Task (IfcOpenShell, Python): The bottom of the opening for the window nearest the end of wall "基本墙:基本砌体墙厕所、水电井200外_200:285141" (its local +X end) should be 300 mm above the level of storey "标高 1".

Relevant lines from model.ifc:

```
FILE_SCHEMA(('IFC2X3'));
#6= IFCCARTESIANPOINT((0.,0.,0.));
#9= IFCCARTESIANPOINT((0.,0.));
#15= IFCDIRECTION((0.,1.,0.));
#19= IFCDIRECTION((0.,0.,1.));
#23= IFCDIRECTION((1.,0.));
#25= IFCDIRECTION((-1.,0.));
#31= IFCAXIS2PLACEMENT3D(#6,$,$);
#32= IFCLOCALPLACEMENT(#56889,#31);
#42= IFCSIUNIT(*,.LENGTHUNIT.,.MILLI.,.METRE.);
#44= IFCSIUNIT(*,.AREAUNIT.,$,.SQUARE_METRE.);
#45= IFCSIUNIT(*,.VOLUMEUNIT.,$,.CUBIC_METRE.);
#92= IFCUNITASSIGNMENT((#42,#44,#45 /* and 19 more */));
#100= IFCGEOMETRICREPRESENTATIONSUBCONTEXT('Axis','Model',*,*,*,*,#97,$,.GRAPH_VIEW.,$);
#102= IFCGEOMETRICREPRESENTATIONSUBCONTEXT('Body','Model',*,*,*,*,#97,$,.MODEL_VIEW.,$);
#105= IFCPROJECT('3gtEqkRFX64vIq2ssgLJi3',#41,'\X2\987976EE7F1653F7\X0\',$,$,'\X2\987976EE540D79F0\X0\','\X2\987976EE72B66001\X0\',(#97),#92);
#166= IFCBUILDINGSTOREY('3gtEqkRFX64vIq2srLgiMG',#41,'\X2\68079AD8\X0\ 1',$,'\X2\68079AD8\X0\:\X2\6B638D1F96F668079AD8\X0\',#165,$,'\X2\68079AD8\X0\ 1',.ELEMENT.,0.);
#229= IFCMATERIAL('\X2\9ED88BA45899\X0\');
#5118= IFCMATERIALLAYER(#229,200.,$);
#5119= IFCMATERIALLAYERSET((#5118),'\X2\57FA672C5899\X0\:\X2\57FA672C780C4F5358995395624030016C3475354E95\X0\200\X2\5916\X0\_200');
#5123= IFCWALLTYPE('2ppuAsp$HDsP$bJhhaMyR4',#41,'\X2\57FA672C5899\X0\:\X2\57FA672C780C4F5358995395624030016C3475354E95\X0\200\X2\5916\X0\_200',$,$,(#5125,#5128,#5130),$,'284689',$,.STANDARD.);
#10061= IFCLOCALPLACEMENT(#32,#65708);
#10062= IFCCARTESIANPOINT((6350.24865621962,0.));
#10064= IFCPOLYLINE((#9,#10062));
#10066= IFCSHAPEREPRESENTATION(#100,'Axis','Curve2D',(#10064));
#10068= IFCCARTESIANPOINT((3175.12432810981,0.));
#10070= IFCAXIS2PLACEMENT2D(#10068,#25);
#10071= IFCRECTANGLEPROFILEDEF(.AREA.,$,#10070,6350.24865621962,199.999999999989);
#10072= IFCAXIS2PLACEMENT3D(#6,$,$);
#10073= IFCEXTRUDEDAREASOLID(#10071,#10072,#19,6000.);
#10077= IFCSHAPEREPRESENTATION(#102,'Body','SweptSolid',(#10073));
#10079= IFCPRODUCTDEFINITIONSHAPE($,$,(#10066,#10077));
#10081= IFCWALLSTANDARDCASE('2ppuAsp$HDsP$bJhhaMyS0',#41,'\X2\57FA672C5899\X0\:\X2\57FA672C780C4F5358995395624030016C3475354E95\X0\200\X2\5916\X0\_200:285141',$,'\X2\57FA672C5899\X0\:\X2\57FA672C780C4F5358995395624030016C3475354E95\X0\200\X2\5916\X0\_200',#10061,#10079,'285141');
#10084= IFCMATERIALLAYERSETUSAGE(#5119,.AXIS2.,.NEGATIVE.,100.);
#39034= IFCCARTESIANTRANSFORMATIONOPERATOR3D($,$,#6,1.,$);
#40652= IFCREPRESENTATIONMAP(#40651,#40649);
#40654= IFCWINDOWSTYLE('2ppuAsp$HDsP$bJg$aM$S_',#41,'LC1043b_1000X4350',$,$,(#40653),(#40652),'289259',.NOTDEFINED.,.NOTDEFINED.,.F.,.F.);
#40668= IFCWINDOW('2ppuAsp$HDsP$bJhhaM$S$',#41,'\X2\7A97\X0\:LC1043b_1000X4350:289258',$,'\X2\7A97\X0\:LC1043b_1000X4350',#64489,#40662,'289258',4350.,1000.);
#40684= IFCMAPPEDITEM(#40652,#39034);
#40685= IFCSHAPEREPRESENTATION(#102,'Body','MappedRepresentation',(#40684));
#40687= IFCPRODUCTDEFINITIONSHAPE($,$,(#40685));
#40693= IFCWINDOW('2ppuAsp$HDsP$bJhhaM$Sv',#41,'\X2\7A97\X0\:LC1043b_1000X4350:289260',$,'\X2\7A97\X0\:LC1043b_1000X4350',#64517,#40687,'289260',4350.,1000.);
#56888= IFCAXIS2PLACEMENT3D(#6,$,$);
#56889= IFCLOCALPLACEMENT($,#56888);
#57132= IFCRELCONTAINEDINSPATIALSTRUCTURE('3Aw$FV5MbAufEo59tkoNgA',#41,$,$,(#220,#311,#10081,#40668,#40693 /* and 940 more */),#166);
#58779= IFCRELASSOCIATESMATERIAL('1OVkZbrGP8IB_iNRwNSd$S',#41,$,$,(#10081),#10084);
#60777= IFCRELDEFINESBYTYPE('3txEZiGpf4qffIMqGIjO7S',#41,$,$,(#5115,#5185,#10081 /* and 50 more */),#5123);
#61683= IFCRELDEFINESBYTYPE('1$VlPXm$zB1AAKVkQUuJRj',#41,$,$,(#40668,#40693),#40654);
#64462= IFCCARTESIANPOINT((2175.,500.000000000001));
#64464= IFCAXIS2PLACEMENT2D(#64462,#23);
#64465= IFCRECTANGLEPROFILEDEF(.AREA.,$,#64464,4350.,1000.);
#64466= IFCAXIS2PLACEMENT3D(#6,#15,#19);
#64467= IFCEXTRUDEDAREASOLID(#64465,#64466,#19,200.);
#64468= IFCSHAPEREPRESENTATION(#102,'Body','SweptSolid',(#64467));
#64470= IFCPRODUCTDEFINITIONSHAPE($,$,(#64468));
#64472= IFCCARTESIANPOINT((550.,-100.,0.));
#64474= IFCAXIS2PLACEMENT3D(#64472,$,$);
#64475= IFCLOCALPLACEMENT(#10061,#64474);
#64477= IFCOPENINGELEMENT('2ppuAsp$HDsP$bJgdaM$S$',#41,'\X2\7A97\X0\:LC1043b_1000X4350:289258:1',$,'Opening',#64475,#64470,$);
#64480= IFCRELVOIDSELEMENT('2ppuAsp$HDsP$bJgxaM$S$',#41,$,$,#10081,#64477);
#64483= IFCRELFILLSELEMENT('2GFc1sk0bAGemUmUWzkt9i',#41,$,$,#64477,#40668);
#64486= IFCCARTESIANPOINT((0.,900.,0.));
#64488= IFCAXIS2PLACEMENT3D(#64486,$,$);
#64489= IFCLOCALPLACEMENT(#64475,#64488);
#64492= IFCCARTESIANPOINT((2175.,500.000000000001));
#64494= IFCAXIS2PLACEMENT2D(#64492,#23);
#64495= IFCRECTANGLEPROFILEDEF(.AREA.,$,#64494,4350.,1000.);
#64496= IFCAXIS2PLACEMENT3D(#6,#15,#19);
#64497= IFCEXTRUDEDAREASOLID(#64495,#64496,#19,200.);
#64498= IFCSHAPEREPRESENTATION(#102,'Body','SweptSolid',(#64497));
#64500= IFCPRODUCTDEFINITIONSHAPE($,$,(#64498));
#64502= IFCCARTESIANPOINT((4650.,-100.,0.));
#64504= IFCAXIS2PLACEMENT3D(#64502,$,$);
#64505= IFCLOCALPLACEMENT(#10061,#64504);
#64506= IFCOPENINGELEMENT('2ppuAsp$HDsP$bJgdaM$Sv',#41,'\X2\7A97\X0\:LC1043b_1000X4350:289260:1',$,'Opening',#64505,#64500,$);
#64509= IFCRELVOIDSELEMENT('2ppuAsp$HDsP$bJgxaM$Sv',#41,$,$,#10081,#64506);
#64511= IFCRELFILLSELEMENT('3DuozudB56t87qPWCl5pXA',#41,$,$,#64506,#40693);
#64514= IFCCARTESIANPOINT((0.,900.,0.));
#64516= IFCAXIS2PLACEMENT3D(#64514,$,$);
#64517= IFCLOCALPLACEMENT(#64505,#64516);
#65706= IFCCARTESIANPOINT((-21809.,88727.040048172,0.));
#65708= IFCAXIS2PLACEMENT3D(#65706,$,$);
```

```python
import numpy as np
import ifcopenshell
import ifcopenshell.api.geometry
import ifcopenshell.geom
import ifcopenshell.util.element
import ifcopenshell.util.placement
import ifcopenshell.util.shape
import ifcopenshell.util.unit

model = ifcopenshell.open("model.ifc")
unit_scale = ifcopenshell.util.unit.calculate_unit_scale(model)

window = model.by_guid("2ppuAsp$HDsP$bJhhaM$Sv")
opening = window.FillsVoids[0].RelatingOpeningElement
storey = ifcopenshell.util.element.get_container(window, ifc_class="IfcBuildingStorey")
level = ifcopenshell.util.placement.get_local_placement(storey.ObjectPlacement)[2, 3]

# The opening's origin need not be at the sill, so measure its lowest point.
shape = ifcopenshell.geom.create_shape(ifcopenshell.geom.settings(), opening)
bottom = ifcopenshell.util.shape.get_shape_bottom_elevation(shape, shape.geometry) / unit_scale
dz = level + 0.3 / unit_scale - bottom

shift = np.array([0.0, 0.0, dz])
# The window is placed relative to its opening, so it follows when the opening moves.
matrix = ifcopenshell.util.placement.get_local_placement(opening.ObjectPlacement)
matrix[:3, 3] += shift
ifcopenshell.api.geometry.edit_object_placement(
    model, product=opening, matrix=matrix, is_si=False, should_transform_children=True
)

print(f"moved by {dz * unit_scale:+.3f} m")

model.write("model_updated.ifc")
```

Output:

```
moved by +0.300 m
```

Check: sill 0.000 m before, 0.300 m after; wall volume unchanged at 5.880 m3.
